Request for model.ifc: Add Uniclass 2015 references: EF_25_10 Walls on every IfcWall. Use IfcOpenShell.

First a look at what the model holds.

```python
import ifcopenshell

model = ifcopenshell.open("model.ifc")
print(model.schema)
print("classifications:", [c.Name for c in model.by_type("IfcClassification")])
for ifc_class in ("IfcDoor", "IfcRoof", "IfcStair", "IfcWall", "IfcWindow"):
    print(ifc_class, len(model.by_type(ifc_class)))
```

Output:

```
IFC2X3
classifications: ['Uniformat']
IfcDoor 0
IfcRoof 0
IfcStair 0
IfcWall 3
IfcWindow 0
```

```python
import ifcopenshell
import ifcopenshell.api.classification

model = ifcopenshell.open("model.ifc")

# IFC2X3 requires Source and Edition and has no link from the project to the system.
system = model.create_entity("IfcClassification", Source="NBS", Edition="2015", Name="Uniclass 2015")

codes = {
    "IfcWall": ("EF_25_10", "Walls"),
}
for ifc_class, (code, name) in codes.items():
    products = model.by_type(ifc_class)
    ifcopenshell.api.classification.add_reference(
        model, products=products, classification=system, identification=code, name=name
    )
    print(code, len(products))

model.write("model_updated.ifc")
```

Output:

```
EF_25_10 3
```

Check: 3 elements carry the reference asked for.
